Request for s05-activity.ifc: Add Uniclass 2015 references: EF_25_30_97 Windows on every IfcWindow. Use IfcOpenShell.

First a look at what the model holds.

```python
import ifcopenshell

model = ifcopenshell.open("s05-activity.ifc")
print(model.schema)
print("classifications:", [c.Name for c in model.by_type("IfcClassification")])
for ifc_class in ("IfcDoor", "IfcRoof", "IfcStair", "IfcWall", "IfcWindow"):
    print(ifc_class, len(model.by_type(ifc_class)))
```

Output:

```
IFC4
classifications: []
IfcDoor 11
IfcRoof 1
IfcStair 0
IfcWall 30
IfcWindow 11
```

```python
import ifcopenshell
import ifcopenshell.api.classification

model = ifcopenshell.open("s05-activity.ifc")

system = ifcopenshell.api.classification.add_classification(model, classification="Uniclass 2015")

codes = {
    "IfcWindow": ("EF_25_30_97", "Windows"),
}
for ifc_class, (code, name) in codes.items():
    products = model.by_type(ifc_class)
    ifcopenshell.api.classification.add_reference(
        model, products=products, classification=system, identification=code, name=name
    )
    print(code, len(products))

model.write("s05-activity_rev.ifc")
```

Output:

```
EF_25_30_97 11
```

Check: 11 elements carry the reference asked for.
